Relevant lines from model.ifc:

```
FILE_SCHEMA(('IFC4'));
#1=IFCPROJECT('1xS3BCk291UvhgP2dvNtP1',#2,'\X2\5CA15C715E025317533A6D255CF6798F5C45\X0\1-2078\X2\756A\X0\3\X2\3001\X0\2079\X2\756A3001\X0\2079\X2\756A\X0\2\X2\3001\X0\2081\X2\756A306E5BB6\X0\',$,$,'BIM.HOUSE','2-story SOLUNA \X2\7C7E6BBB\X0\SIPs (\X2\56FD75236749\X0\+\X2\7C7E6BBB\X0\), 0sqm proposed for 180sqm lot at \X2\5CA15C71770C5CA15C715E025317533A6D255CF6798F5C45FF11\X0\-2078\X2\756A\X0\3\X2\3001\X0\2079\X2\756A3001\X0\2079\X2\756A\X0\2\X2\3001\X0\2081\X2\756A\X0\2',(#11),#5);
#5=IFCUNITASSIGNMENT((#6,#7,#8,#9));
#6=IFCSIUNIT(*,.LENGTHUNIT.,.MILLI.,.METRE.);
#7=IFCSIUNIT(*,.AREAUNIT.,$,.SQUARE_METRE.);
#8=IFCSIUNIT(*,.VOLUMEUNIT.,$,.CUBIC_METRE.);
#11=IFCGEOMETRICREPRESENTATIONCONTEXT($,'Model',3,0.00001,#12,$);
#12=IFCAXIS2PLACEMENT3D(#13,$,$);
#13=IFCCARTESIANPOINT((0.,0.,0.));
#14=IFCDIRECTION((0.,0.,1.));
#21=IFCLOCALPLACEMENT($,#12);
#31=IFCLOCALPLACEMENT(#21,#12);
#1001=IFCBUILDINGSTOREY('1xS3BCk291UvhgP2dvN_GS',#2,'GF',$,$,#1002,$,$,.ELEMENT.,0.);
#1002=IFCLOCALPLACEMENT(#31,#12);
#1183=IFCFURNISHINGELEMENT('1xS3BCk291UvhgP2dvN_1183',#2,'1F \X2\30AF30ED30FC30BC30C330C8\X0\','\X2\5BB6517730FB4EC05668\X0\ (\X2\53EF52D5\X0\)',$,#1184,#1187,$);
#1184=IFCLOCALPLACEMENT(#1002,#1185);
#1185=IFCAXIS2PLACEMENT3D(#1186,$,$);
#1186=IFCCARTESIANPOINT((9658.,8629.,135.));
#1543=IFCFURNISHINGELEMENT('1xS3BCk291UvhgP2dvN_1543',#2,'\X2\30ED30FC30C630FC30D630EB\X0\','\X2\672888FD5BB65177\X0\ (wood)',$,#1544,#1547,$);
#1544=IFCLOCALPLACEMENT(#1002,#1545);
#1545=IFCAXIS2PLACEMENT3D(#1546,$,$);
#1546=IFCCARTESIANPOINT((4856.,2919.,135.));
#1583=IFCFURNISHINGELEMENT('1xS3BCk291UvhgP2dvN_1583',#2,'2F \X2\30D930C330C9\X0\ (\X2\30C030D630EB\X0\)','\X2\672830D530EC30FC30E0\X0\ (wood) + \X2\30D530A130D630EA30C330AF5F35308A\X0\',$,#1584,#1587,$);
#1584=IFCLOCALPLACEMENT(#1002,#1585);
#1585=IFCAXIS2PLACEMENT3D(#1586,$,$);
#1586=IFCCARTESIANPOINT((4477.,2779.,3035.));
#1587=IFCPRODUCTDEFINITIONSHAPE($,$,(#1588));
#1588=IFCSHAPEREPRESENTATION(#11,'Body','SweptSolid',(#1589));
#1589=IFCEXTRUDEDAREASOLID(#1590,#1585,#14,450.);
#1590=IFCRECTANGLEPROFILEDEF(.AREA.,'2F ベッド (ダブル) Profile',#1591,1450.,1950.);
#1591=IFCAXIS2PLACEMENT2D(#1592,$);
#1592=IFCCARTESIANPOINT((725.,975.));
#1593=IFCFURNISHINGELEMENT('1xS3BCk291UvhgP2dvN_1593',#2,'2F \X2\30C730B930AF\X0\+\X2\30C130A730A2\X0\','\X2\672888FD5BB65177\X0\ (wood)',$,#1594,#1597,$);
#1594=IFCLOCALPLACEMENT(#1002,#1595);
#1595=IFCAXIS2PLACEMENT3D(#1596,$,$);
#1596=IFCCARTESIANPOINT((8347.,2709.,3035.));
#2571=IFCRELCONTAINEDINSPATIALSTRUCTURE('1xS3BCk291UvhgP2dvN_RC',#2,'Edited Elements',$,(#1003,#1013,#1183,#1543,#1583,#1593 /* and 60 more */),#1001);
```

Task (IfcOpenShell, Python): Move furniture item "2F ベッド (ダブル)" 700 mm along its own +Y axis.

```python
import ifcopenshell
import ifcopenshell.api.geometry
import ifcopenshell.util.placement

model = ifcopenshell.open("model.ifc")

item = model.by_guid("1xS3BCk291UvhgP2dvN_1583")
matrix = ifcopenshell.util.placement.get_local_placement(item.ObjectPlacement)
matrix[:3, 3] += matrix[:3, 1] * 700.0
ifcopenshell.api.geometry.edit_object_placement(model, product=item, matrix=matrix, is_si=False)

print(ifcopenshell.util.placement.get_local_placement(item.ObjectPlacement).round(3) + 0.0)

model.write("model_updated.ifc")
```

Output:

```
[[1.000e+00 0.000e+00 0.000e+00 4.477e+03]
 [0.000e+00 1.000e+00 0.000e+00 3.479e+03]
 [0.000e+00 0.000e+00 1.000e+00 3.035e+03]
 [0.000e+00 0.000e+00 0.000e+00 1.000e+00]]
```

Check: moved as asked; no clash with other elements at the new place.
